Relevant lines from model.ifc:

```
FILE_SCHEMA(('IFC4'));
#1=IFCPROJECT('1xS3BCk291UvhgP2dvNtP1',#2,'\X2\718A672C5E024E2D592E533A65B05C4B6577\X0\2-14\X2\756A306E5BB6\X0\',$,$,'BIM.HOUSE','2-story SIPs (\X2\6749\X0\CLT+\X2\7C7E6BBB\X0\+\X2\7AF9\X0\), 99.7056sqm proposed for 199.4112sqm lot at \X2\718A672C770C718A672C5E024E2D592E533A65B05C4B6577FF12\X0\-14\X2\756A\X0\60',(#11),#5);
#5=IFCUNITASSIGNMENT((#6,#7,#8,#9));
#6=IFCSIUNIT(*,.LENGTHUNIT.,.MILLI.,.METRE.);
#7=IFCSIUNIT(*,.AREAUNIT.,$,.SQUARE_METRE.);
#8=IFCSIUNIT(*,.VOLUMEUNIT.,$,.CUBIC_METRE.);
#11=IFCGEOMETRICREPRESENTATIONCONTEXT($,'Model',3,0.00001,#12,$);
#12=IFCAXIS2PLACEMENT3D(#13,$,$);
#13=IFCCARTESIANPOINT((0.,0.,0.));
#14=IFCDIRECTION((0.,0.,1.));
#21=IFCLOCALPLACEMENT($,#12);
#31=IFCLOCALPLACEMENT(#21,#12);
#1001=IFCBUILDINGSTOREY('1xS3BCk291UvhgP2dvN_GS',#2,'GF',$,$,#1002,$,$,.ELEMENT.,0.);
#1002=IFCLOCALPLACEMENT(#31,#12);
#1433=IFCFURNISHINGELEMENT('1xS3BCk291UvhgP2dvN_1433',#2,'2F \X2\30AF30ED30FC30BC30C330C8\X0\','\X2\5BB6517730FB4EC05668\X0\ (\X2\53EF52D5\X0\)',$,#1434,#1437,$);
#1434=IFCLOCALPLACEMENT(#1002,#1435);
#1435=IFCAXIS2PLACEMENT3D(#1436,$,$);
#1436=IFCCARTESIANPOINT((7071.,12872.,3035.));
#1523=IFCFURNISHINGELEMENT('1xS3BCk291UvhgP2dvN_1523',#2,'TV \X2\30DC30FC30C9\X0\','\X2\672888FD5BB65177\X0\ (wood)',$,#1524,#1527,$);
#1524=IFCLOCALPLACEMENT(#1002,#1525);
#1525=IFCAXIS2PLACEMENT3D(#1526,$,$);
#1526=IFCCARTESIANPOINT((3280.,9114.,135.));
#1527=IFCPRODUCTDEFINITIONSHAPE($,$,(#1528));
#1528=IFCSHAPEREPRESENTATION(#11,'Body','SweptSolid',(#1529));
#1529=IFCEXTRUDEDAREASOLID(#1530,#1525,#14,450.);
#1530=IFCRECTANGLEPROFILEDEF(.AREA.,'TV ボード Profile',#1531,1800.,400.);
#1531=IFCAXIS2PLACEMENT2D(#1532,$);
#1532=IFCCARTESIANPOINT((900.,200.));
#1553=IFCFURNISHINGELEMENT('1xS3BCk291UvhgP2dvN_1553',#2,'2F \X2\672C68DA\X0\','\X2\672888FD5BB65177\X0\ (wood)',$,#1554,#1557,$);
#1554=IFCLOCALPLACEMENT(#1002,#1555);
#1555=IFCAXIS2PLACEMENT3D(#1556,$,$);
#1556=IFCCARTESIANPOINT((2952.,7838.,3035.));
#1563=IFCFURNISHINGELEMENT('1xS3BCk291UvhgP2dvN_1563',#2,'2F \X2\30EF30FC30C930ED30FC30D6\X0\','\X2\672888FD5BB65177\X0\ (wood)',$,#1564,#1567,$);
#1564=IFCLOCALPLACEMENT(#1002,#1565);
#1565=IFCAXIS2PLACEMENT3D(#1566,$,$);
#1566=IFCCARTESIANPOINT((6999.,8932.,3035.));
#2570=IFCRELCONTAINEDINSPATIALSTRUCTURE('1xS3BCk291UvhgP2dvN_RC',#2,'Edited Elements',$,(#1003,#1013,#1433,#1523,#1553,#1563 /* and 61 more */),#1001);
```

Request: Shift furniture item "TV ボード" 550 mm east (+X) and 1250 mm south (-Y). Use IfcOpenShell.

```python
import ifcopenshell
import ifcopenshell.api.geometry
import ifcopenshell.util.placement
import ifcopenshell.util.unit

model = ifcopenshell.open("model.ifc")
unit_scale = ifcopenshell.util.unit.calculate_unit_scale(model)

item = model.by_guid("1xS3BCk291UvhgP2dvN_1523")
matrix = ifcopenshell.util.placement.get_local_placement(item.ObjectPlacement)
matrix[0, 3] += 0.55 / unit_scale
matrix[1, 3] -= 1.25 / unit_scale
ifcopenshell.api.geometry.edit_object_placement(model, product=item, matrix=matrix, is_si=False)

print(ifcopenshell.util.placement.get_local_placement(item.ObjectPlacement).round(3) + 0.0)

model.write("model_updated.ifc")
```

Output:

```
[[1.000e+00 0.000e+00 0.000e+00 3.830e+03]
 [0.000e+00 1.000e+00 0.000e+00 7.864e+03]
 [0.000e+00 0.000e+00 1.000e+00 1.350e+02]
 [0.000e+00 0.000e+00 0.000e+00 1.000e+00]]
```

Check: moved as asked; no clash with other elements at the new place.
